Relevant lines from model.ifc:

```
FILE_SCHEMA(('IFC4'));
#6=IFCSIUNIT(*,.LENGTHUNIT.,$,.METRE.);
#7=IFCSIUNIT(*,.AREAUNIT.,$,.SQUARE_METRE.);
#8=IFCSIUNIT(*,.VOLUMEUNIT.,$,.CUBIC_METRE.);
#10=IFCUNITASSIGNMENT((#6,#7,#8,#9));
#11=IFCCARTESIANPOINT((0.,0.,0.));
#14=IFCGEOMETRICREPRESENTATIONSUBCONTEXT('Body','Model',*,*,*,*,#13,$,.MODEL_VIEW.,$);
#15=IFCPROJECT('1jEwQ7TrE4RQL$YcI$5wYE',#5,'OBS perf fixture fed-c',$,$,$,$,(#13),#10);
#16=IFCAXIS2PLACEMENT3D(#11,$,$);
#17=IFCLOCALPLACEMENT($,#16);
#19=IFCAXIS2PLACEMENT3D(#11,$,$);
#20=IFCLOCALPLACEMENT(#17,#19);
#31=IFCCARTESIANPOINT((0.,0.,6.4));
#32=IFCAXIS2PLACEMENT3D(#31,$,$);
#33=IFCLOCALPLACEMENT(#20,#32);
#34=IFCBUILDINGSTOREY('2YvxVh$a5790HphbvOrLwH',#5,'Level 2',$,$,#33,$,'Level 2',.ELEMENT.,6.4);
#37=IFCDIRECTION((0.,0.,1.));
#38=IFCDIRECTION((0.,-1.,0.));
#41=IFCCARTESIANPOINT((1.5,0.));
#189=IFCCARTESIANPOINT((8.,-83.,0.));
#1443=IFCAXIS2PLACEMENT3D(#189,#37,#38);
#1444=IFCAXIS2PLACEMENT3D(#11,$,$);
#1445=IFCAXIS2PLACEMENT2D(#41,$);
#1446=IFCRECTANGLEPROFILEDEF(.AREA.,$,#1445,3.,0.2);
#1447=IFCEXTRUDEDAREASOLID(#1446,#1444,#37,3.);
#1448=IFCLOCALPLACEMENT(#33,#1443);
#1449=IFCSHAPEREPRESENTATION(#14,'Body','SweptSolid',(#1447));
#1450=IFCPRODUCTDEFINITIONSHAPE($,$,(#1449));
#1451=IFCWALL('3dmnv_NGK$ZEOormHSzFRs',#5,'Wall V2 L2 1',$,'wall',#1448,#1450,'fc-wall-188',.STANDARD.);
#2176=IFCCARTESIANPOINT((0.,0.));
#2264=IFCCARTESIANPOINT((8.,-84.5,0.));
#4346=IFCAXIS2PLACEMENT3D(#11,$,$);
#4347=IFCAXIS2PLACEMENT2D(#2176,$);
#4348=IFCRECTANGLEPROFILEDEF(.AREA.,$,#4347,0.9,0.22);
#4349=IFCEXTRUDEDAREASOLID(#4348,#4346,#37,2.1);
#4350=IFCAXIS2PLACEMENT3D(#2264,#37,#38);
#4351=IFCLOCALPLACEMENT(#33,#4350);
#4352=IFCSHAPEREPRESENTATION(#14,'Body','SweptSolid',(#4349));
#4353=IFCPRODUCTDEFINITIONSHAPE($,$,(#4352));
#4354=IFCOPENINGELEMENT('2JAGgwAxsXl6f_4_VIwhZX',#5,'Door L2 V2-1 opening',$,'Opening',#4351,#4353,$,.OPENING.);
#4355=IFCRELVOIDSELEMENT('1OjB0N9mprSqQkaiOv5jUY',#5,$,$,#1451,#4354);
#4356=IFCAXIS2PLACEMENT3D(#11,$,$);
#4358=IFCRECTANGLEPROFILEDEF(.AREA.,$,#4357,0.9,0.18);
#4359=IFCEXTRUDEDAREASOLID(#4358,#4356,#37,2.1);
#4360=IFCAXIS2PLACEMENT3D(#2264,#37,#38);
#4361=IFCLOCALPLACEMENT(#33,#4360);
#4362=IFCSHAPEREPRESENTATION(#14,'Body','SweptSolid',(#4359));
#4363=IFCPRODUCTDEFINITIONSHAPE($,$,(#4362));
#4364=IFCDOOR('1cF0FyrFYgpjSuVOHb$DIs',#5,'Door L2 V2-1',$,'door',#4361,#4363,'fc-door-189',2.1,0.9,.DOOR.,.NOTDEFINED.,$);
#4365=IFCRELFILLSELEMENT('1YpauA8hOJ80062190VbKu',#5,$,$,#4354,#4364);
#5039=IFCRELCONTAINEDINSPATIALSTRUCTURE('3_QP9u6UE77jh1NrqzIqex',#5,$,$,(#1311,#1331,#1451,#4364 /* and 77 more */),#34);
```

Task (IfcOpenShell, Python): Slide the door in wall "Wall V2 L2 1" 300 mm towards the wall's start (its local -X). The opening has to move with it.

```python
import ifcopenshell
import ifcopenshell.api.geometry
import ifcopenshell.util.placement

model = ifcopenshell.open("model.ifc")

door = model.by_guid("1cF0FyrFYgpjSuVOHb$DIs")
opening = door.FillsVoids[0].RelatingOpeningElement
wall = opening.VoidsElements[0].RelatingBuildingElement

wall_matrix = ifcopenshell.util.placement.get_local_placement(wall.ObjectPlacement)
shift = wall_matrix[:3, 0] * -0.3
before = ifcopenshell.util.placement.get_local_placement(door.ObjectPlacement)[:3, 3].copy()

# The door is not placed relative to its opening, so move both.
for product in (opening, door):
    matrix = ifcopenshell.util.placement.get_local_placement(product.ObjectPlacement)
    matrix[:3, 3] += shift
    ifcopenshell.api.geometry.edit_object_placement(model, product=product, matrix=matrix, is_si=False)

after = ifcopenshell.util.placement.get_local_placement(door.ObjectPlacement)[:3, 3]
print("door moved by", (after - before).round(3) + 0.0)

model.write("model_edited.ifc")
```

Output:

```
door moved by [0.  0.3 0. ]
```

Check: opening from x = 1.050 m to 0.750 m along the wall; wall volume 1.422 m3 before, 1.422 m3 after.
